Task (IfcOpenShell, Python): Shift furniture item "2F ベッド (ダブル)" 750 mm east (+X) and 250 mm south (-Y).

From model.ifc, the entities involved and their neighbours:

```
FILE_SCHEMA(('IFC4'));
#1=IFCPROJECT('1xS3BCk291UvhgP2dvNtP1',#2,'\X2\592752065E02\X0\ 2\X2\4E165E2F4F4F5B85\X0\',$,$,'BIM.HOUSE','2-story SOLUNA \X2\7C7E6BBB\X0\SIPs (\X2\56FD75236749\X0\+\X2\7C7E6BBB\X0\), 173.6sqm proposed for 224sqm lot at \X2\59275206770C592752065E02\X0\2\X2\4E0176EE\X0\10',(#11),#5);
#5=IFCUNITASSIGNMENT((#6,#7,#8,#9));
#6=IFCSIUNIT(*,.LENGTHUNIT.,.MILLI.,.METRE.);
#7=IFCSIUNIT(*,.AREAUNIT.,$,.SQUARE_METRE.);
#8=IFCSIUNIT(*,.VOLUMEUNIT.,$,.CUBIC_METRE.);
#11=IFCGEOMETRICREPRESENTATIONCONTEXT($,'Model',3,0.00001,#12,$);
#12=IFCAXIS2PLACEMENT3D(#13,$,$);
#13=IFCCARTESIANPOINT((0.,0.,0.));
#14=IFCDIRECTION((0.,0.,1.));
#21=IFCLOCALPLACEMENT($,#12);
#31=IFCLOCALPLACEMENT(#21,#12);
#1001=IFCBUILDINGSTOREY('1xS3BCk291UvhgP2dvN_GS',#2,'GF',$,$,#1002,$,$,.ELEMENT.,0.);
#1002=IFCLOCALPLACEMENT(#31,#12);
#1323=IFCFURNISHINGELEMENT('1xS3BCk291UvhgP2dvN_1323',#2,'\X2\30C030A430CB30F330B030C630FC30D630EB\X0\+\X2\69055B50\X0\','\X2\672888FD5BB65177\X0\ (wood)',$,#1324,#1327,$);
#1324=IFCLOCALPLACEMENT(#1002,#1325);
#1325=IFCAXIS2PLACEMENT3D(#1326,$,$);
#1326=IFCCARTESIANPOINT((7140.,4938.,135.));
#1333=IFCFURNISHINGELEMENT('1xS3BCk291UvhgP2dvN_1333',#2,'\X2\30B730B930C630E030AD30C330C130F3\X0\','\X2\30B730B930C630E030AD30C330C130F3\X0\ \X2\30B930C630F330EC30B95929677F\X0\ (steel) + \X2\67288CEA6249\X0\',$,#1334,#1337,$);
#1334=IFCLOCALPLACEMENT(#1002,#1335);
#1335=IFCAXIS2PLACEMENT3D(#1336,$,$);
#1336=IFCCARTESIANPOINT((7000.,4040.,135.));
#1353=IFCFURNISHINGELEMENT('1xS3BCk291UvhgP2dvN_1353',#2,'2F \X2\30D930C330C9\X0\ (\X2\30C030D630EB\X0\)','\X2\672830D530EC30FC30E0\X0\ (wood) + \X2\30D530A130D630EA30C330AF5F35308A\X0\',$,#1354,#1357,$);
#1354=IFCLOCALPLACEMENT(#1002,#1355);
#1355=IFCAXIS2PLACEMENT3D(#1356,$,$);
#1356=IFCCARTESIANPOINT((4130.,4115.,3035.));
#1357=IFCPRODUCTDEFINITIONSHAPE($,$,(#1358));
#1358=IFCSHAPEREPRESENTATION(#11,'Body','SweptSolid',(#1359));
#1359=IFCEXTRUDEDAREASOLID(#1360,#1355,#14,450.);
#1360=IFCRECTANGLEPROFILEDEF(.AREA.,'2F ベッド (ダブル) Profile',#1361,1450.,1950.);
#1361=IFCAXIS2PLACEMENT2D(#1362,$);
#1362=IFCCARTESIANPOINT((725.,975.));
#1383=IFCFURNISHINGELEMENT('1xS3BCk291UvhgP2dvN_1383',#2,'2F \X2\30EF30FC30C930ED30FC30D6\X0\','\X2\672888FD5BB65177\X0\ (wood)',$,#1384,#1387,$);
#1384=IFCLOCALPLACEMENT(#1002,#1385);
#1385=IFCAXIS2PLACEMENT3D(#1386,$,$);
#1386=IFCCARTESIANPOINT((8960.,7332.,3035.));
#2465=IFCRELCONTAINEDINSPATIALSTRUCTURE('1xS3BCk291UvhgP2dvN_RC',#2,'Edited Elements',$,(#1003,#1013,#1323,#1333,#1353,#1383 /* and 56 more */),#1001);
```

```python
import ifcopenshell
import ifcopenshell.api.geometry
import ifcopenshell.util.placement
import ifcopenshell.util.unit

model = ifcopenshell.open("model.ifc")
unit_scale = ifcopenshell.util.unit.calculate_unit_scale(model)

item = model.by_guid("1xS3BCk291UvhgP2dvN_1353")
matrix = ifcopenshell.util.placement.get_local_placement(item.ObjectPlacement)
matrix[0, 3] += 0.75 / unit_scale
matrix[1, 3] -= 0.25 / unit_scale
ifcopenshell.api.geometry.edit_object_placement(model, product=item, matrix=matrix, is_si=False)

print(ifcopenshell.util.placement.get_local_placement(item.ObjectPlacement).round(3) + 0.0)

model.write("model_rev.ifc")
```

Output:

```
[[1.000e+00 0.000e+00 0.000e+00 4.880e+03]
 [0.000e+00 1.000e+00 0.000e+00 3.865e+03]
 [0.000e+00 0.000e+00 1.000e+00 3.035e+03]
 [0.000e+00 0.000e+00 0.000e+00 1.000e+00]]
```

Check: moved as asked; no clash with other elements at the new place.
